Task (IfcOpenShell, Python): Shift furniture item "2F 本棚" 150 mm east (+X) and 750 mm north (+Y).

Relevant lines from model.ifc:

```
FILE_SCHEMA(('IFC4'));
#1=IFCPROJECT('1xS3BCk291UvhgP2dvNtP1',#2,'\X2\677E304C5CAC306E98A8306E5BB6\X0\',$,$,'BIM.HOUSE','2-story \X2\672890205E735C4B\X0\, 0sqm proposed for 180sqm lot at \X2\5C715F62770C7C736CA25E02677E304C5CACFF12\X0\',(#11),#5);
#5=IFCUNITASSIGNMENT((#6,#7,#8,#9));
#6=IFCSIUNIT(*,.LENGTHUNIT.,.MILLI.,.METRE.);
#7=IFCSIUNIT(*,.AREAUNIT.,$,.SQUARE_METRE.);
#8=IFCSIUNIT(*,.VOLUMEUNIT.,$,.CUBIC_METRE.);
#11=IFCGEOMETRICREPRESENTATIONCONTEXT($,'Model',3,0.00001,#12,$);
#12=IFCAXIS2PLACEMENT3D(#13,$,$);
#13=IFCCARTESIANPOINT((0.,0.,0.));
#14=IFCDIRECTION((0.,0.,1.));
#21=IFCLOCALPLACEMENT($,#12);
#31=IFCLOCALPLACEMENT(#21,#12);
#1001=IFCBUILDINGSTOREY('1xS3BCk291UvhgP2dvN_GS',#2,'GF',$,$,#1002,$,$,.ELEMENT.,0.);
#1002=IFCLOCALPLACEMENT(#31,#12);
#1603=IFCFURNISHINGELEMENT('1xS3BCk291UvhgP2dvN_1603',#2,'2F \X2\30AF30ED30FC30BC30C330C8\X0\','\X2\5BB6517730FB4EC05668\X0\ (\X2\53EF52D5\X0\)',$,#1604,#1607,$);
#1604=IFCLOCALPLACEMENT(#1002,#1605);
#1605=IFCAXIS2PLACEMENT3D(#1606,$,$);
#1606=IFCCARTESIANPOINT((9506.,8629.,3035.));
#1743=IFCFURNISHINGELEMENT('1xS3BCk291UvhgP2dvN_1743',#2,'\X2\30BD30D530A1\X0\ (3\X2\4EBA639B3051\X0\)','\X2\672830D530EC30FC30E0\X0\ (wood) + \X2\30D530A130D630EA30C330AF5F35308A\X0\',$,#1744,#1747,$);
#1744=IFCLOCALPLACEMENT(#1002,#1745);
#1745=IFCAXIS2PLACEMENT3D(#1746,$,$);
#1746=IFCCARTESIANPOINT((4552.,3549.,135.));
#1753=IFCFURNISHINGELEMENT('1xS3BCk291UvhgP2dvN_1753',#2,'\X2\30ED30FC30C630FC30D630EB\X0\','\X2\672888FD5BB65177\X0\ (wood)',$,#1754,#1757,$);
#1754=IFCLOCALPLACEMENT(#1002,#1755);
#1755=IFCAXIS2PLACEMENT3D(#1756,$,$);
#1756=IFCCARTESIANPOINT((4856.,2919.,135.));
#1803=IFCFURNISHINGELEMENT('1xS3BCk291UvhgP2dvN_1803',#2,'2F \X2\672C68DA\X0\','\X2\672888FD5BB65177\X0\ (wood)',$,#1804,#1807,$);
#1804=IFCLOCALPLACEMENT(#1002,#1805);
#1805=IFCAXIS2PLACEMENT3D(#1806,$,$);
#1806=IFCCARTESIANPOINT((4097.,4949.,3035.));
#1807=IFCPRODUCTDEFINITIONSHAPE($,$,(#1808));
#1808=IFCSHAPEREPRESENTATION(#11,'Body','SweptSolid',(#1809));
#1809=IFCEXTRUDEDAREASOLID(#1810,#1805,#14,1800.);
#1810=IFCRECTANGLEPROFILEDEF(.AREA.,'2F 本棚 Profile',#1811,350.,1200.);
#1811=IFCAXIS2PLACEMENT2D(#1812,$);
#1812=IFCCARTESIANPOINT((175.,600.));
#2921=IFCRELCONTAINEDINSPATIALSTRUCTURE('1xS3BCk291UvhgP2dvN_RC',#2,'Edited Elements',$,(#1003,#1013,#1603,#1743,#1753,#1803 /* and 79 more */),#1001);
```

```python
import ifcopenshell
import ifcopenshell.api.geometry
import ifcopenshell.util.placement

model = ifcopenshell.open("model.ifc")

item = model.by_guid("1xS3BCk291UvhgP2dvN_1803")
matrix = ifcopenshell.util.placement.get_local_placement(item.ObjectPlacement)
matrix[0, 3] += 150.0
matrix[1, 3] += 750.0
ifcopenshell.api.geometry.edit_object_placement(model, product=item, matrix=matrix, is_si=False)

print(ifcopenshell.util.placement.get_local_placement(item.ObjectPlacement).round(3) + 0.0)

model.write("model_rev.ifc")
```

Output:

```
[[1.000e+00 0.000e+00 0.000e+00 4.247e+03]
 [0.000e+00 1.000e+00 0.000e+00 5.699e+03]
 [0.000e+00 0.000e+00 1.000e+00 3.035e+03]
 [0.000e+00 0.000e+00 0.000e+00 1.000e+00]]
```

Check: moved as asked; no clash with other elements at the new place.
